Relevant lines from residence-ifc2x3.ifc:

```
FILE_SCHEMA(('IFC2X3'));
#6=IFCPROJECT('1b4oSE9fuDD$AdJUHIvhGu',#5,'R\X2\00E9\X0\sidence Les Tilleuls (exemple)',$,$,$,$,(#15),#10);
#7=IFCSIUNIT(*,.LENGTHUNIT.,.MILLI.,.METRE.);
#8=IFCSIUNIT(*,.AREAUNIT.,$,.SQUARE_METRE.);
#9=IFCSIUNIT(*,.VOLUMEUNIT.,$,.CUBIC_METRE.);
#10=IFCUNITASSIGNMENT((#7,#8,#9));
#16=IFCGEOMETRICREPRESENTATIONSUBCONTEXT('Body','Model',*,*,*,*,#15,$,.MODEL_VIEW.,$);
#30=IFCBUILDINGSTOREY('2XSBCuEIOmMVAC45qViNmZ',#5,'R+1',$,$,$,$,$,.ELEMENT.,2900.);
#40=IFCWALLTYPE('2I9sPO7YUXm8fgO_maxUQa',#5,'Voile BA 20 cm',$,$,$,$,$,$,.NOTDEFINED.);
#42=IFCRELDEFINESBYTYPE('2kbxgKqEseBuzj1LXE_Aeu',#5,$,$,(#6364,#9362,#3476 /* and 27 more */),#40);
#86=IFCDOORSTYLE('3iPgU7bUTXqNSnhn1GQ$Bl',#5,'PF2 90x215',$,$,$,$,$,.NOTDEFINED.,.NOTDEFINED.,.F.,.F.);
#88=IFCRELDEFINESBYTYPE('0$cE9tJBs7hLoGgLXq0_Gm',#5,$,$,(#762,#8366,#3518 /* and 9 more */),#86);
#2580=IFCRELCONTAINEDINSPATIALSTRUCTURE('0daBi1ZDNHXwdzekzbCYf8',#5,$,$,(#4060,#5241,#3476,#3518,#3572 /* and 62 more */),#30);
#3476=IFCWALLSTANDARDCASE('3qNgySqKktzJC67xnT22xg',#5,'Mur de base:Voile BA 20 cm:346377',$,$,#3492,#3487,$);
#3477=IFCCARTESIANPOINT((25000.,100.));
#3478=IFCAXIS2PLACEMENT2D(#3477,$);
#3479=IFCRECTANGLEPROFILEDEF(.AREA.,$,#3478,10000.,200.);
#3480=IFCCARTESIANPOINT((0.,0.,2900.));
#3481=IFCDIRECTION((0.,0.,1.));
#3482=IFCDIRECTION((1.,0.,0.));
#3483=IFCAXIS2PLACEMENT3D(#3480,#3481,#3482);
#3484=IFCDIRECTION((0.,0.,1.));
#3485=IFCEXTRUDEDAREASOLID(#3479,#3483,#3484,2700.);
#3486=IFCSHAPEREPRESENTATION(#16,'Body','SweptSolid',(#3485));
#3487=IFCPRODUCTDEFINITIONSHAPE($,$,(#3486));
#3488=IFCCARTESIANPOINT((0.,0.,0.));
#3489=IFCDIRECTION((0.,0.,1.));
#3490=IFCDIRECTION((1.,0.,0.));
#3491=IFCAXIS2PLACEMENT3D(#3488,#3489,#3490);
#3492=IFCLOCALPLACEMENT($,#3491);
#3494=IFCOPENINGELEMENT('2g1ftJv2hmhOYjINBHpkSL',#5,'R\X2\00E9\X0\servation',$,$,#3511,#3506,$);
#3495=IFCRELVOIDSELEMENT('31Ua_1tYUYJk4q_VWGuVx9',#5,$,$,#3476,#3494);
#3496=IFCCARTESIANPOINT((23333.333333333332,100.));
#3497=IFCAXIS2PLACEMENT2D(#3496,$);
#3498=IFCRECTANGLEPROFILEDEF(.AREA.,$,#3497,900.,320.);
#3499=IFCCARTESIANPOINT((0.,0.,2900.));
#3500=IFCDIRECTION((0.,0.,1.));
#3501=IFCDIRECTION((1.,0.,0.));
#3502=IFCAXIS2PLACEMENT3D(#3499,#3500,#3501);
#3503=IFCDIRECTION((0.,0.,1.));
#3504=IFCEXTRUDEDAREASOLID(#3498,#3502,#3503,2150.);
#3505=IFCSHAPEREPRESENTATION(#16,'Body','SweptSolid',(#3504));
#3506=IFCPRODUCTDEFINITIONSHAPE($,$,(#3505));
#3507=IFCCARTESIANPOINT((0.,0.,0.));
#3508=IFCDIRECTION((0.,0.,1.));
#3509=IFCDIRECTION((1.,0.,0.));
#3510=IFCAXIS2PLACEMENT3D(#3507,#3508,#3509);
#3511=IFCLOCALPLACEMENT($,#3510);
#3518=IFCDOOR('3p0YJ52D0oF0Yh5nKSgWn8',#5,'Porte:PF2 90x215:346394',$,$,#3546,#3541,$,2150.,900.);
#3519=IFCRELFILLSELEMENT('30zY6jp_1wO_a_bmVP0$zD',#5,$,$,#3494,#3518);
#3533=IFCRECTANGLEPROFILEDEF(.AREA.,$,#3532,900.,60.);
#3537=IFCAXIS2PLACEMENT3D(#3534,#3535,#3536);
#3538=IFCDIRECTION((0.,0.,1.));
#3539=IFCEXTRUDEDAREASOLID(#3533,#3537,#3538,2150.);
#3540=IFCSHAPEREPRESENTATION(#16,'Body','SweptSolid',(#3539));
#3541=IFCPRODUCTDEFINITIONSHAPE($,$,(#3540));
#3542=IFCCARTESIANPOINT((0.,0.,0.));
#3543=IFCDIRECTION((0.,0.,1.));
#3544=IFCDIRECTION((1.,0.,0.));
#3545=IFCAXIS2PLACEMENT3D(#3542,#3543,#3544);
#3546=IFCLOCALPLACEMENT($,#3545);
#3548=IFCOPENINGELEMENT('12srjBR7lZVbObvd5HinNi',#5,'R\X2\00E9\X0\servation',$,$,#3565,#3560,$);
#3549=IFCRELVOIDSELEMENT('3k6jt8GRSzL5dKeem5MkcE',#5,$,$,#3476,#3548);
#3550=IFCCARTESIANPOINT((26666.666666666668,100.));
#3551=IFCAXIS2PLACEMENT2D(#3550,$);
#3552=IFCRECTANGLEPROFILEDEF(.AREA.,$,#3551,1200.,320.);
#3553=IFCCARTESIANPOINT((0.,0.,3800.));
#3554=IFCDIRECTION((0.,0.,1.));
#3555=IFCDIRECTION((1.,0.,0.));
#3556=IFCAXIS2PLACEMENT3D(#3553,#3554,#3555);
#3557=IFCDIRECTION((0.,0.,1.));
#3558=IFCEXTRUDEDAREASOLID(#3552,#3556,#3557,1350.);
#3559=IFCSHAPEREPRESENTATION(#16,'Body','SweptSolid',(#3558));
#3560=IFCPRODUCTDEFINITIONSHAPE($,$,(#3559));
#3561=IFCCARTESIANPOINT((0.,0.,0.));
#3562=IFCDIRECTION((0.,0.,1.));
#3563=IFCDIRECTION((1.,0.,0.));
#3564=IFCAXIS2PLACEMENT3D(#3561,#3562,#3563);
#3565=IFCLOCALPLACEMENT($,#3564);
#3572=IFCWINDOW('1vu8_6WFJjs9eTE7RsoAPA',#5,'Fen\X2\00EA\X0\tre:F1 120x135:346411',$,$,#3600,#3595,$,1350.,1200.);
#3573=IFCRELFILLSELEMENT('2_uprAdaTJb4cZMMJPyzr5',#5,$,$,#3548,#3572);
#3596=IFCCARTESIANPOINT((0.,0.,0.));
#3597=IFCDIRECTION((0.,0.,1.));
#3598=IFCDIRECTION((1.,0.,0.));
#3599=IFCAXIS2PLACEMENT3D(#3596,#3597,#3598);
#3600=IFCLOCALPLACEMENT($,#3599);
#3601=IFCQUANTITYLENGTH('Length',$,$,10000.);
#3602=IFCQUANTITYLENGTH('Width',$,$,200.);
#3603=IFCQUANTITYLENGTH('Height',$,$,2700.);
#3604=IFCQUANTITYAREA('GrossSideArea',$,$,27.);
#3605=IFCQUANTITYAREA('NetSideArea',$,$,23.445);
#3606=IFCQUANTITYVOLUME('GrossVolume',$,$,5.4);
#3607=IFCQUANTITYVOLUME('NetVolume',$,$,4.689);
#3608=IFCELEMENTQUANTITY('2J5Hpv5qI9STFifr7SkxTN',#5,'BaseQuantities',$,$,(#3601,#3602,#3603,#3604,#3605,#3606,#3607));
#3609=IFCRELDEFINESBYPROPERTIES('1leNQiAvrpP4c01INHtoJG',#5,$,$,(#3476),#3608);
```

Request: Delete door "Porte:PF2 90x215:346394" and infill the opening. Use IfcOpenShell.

```python
import ifcopenshell
import ifcopenshell.api.feature
import ifcopenshell.api.pset
import ifcopenshell.api.root
import ifcopenshell.geom
import ifcopenshell.util.element
import ifcopenshell.util.shape
import ifcopenshell.util.unit

model = ifcopenshell.open("residence-ifc2x3.ifc")
area_scale = ifcopenshell.util.unit.calculate_unit_scale(model, "AREAUNIT")
volume_scale = ifcopenshell.util.unit.calculate_unit_scale(model, "VOLUMEUNIT")
settings = ifcopenshell.geom.settings()


def volume(element):
    """Net volume in cubic metres, openings subtracted."""
    shape = ifcopenshell.geom.create_shape(settings, element)
    return ifcopenshell.util.shape.get_volume(shape.geometry)


door = model.by_guid("3p0YJ52D0oF0Yh5nKSgWn8")
opening = door.FillsVoids[0].RelatingOpeningElement
wall = opening.VoidsElements[0].RelatingBuildingElement
before = volume(wall)

ifcopenshell.api.root.remove_product(model, product=door)
ifcopenshell.api.feature.remove_feature(model, feature=opening)

after = volume(wall)
thickness = 0.2  # wall thickness in metres

# Update the wall's stored quantities.
qto = model.by_id(ifcopenshell.util.element.get_pset(wall, "BaseQuantities", should_inherit=False)["id"])
ifcopenshell.api.pset.edit_qto(model, qto=qto, properties={
    "NetSideArea": after / thickness / area_scale,
    "NetVolume": after / volume_scale,
})

print(f"wall volume {before:.3f} -> {after:.3f} m3")

model.write("residence-ifc2x3_updated.ifc")
```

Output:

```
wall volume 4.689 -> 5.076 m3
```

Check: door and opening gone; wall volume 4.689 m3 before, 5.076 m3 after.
